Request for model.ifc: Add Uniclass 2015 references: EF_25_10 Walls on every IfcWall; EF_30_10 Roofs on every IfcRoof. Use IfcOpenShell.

First a look at what the model holds.

```python
import ifcopenshell

model = ifcopenshell.open("model.ifc")
print(model.schema)
print("classifications:", [c.Name for c in model.by_type("IfcClassification")])
for ifc_class in ("IfcDoor", "IfcRoof", "IfcStair", "IfcWall", "IfcWindow"):
    print(ifc_class, len(model.by_type(ifc_class)))
```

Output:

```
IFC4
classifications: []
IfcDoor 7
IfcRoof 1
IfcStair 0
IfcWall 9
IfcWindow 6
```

```python
import ifcopenshell
import ifcopenshell.api.classification

model = ifcopenshell.open("model.ifc")

system = ifcopenshell.api.classification.add_classification(model, classification="Uniclass 2015")

codes = {
    "IfcWall": ("EF_25_10", "Walls"),
    "IfcRoof": ("EF_30_10", "Roofs"),
}
for ifc_class, (code, name) in codes.items():
    products = model.by_type(ifc_class)
    ifcopenshell.api.classification.add_reference(
        model, products=products, classification=system, identification=code, name=name
    )
    print(code, len(products))

model.write("model_updated.ifc")
```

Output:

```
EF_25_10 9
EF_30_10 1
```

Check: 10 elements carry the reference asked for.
